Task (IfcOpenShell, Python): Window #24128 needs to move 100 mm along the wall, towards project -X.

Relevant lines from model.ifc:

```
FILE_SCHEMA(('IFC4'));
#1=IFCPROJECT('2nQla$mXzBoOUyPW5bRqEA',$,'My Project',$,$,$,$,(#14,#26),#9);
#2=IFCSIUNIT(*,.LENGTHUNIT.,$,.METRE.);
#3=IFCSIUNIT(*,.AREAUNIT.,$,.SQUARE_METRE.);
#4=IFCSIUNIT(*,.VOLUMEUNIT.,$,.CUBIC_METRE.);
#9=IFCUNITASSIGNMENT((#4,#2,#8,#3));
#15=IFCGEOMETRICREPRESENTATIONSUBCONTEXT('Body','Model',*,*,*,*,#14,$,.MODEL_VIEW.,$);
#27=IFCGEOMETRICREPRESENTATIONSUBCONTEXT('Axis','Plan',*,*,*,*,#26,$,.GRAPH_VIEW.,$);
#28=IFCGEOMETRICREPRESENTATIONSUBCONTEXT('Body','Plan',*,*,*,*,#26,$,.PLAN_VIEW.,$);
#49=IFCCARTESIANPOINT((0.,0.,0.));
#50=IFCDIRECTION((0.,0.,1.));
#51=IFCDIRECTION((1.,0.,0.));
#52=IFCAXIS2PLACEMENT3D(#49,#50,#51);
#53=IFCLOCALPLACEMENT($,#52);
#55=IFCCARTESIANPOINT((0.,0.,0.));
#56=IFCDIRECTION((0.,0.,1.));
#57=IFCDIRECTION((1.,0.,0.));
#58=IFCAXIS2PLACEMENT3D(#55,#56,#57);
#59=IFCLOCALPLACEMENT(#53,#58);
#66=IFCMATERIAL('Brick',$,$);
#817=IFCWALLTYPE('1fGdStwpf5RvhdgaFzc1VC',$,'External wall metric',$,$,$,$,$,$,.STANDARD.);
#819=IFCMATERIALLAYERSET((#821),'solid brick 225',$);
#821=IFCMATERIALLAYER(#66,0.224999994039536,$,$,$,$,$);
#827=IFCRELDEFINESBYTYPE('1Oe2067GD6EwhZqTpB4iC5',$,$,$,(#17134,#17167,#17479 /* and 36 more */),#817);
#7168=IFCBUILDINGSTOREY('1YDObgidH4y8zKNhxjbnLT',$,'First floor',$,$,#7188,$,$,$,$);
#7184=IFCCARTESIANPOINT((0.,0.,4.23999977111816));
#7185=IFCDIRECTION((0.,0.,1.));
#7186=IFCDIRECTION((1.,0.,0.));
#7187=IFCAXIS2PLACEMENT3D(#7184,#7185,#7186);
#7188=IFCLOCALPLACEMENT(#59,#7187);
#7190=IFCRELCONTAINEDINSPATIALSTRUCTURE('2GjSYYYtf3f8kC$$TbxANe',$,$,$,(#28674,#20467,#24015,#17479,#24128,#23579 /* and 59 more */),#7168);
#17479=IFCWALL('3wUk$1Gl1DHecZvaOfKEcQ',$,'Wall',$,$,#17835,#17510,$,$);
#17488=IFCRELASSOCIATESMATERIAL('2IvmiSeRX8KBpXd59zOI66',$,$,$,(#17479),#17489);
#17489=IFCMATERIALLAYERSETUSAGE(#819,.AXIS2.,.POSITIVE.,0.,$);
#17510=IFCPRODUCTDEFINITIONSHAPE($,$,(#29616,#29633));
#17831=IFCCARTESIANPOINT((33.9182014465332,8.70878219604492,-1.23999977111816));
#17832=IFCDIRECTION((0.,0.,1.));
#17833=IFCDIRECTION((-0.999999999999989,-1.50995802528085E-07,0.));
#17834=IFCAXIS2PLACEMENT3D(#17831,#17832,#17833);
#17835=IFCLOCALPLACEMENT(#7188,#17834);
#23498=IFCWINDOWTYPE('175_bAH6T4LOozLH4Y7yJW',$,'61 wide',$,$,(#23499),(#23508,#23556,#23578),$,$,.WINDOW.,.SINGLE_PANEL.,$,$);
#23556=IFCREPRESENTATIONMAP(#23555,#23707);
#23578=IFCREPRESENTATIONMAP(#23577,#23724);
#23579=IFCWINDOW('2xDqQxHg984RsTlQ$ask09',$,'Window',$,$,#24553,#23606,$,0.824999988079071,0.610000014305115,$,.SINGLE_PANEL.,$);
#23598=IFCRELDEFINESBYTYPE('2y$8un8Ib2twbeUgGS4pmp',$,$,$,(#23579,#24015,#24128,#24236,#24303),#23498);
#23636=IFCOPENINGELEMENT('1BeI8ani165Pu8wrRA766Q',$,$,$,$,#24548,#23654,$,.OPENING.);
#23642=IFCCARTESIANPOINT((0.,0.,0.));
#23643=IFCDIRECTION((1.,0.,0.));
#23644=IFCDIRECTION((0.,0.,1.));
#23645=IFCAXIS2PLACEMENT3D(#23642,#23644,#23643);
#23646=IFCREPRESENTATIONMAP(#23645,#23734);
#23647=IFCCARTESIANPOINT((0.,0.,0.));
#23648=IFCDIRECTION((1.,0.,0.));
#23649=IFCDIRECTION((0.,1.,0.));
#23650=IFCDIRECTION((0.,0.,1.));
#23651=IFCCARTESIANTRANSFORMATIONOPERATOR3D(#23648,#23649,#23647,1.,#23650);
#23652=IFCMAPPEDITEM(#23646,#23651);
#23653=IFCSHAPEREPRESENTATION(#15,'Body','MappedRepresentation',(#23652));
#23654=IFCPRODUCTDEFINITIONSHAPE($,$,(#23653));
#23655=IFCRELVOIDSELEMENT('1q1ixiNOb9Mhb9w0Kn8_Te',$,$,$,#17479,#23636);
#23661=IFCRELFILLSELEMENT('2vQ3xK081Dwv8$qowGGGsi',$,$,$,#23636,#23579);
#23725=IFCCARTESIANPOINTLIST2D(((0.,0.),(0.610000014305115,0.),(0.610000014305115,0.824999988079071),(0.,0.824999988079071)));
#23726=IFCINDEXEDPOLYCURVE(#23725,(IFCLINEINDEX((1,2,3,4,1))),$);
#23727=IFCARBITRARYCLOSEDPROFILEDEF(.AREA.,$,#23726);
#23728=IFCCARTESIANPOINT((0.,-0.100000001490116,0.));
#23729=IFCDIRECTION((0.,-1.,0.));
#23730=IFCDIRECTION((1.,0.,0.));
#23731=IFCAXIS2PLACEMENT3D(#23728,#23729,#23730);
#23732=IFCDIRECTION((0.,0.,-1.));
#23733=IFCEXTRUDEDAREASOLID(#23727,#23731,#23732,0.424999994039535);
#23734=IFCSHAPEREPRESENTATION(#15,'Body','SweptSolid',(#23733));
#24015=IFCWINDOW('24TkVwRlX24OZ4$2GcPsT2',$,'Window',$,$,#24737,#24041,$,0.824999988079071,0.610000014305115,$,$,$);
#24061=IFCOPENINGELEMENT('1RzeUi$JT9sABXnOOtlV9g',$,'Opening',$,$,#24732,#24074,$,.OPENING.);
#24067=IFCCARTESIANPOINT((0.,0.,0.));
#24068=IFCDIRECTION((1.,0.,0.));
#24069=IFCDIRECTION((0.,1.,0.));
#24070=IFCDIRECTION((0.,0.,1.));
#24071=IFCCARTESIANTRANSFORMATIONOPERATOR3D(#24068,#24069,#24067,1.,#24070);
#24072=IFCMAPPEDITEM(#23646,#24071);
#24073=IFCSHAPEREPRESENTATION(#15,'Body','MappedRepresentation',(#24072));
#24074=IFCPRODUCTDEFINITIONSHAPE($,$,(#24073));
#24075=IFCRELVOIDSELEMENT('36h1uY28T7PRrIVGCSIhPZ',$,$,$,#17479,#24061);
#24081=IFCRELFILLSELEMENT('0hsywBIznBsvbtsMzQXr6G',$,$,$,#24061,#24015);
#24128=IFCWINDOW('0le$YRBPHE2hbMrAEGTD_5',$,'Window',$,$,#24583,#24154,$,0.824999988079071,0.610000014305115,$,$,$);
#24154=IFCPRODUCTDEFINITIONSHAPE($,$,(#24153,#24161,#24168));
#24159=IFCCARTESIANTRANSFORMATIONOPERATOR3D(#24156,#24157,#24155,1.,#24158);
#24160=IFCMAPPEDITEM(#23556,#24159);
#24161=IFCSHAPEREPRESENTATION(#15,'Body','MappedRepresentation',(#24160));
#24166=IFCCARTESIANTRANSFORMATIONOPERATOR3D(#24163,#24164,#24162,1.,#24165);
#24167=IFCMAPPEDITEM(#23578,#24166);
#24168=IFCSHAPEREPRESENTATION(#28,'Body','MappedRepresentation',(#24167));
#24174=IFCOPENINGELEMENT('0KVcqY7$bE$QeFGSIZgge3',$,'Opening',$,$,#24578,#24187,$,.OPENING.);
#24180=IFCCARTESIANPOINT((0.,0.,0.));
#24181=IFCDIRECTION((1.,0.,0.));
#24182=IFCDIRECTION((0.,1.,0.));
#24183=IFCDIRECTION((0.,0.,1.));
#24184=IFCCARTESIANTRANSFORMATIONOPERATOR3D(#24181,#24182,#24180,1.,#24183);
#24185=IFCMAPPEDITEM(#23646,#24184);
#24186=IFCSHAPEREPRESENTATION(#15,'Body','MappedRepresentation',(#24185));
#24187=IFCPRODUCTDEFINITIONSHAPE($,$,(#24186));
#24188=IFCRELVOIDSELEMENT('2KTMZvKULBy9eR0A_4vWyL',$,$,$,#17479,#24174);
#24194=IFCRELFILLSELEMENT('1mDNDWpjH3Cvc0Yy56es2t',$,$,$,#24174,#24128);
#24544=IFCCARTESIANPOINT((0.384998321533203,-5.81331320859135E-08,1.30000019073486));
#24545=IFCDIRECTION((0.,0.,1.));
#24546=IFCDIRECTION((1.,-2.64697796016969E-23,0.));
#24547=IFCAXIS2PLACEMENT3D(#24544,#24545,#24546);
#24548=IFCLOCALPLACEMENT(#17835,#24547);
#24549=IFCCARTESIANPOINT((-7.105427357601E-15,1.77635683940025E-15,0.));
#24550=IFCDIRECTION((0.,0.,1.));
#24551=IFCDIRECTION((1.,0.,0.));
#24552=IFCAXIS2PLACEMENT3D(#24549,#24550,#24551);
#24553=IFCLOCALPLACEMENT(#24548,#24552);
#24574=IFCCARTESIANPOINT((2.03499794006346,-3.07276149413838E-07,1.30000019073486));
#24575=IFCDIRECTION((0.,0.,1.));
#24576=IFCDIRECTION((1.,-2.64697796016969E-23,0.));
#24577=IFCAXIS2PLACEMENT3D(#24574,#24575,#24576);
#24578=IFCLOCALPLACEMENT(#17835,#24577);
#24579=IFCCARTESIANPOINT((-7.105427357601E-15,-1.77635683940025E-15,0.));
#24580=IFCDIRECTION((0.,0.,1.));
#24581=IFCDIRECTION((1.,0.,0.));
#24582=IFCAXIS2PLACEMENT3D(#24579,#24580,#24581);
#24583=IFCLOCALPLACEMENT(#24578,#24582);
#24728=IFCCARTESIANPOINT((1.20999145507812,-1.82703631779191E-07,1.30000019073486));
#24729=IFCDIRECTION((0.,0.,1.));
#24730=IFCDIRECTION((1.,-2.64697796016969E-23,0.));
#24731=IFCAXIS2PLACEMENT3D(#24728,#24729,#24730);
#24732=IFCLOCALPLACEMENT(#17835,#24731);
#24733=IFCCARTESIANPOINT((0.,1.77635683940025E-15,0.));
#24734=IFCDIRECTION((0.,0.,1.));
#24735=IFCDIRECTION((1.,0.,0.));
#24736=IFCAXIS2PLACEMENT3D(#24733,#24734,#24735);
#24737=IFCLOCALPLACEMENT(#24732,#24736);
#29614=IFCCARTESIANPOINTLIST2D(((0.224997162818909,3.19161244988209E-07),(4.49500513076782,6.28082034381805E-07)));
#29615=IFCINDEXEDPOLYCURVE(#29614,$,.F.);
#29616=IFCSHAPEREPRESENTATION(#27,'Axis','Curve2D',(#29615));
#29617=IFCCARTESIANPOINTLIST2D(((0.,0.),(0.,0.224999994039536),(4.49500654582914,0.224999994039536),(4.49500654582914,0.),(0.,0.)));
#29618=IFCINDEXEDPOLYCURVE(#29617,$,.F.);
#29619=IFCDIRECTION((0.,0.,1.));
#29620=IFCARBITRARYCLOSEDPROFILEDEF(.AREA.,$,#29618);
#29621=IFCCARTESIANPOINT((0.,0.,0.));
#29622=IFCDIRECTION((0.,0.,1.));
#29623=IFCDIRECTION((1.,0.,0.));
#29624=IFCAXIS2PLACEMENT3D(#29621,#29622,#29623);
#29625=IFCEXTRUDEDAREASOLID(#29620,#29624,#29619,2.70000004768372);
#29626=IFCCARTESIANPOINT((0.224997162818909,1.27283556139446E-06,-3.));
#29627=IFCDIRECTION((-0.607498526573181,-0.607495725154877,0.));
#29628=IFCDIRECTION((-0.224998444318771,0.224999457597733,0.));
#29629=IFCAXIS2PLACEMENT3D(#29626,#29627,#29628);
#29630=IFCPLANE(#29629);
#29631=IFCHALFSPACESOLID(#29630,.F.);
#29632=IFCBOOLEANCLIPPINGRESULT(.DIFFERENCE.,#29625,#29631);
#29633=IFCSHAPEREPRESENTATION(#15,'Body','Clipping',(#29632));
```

```python
import ifcopenshell
import ifcopenshell.api.geometry
import ifcopenshell.util.placement
import ifcopenshell.util.unit

model = ifcopenshell.open("model.ifc")
unit_scale = ifcopenshell.util.unit.calculate_unit_scale(model)

window = model.by_guid("0le$YRBPHE2hbMrAEGTD_5")
opening = window.FillsVoids[0].RelatingOpeningElement
wall = opening.VoidsElements[0].RelatingBuildingElement

wall_matrix = ifcopenshell.util.placement.get_local_placement(wall.ObjectPlacement)
shift = wall_matrix[:3, 0] * 0.1 / unit_scale
before = ifcopenshell.util.placement.get_local_placement(window.ObjectPlacement)[:3, 3].copy()

# The window is placed relative to its opening, so it follows when the opening moves.
matrix = ifcopenshell.util.placement.get_local_placement(opening.ObjectPlacement)
matrix[:3, 3] += shift
ifcopenshell.api.geometry.edit_object_placement(
    model, product=opening, matrix=matrix, is_si=False, should_transform_children=True
)

after = ifcopenshell.util.placement.get_local_placement(window.ObjectPlacement)[:3, 3]
print("window moved by", (after - before).round(3) + 0.0)

model.write("model_v2.ifc")
```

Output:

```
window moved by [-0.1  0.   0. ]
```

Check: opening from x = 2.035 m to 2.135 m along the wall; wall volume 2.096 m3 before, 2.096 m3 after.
